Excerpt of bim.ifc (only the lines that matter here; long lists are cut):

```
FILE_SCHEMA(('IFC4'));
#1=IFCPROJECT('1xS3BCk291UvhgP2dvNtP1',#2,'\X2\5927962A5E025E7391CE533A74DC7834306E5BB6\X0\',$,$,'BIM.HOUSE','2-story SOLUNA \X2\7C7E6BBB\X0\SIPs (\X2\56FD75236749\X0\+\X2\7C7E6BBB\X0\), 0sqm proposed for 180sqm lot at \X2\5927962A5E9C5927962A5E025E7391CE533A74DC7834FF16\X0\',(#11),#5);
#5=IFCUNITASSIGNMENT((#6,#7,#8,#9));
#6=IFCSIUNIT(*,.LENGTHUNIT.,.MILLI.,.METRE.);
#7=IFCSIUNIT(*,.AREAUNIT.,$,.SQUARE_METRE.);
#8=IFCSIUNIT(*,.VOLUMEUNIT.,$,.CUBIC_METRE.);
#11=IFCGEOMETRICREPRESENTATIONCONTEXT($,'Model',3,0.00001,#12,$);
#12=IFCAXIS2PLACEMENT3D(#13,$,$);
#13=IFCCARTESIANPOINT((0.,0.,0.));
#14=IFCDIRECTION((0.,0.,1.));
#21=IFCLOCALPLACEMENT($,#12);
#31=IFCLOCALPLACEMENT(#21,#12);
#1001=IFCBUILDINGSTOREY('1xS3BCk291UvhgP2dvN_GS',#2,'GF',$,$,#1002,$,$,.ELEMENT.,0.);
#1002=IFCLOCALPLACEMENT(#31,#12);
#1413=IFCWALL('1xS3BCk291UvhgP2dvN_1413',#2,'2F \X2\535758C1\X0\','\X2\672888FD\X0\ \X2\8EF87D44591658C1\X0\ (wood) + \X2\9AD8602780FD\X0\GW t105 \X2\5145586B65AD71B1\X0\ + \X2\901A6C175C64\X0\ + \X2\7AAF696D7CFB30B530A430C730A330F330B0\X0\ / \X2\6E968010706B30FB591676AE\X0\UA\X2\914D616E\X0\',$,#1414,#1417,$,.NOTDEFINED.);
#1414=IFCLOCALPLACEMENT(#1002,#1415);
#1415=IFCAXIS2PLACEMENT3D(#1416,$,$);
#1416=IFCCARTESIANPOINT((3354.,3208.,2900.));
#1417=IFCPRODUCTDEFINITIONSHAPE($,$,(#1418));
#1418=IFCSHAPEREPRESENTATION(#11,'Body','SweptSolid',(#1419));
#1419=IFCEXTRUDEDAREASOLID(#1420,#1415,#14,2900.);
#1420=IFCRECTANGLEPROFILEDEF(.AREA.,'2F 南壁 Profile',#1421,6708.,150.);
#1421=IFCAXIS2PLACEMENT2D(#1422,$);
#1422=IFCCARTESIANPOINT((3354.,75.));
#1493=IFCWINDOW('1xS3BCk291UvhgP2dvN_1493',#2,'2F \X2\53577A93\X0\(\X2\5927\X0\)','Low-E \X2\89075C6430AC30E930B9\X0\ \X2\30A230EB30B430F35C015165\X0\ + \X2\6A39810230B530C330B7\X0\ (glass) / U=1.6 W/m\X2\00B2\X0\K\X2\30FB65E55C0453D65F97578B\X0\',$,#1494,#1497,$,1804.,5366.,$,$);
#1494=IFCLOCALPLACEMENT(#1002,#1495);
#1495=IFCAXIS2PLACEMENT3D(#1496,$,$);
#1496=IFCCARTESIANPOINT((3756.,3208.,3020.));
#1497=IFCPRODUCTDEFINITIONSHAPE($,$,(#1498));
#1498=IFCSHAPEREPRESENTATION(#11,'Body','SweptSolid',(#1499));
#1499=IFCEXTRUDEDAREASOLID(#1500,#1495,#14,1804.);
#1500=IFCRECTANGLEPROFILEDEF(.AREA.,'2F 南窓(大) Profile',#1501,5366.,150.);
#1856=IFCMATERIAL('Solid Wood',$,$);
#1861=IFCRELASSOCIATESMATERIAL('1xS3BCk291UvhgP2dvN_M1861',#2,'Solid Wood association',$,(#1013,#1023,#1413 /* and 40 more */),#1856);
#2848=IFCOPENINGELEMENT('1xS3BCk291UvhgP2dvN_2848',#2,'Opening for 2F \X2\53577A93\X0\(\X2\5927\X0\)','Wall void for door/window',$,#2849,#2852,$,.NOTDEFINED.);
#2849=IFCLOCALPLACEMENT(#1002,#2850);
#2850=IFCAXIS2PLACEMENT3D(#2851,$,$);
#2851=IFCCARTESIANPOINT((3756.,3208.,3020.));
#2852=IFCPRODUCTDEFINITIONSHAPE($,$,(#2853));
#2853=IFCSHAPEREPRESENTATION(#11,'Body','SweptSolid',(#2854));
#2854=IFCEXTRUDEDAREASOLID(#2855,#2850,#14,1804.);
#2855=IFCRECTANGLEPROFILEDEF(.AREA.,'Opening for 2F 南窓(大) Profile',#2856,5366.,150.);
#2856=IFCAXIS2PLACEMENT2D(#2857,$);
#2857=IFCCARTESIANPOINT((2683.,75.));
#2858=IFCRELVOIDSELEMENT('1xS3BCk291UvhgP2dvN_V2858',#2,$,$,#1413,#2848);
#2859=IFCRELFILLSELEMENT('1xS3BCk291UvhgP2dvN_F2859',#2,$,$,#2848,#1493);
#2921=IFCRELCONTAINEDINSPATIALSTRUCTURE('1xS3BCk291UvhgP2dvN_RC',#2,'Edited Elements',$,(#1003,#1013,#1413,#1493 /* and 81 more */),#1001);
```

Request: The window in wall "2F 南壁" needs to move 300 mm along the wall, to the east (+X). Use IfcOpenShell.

```python
import ifcopenshell
import ifcopenshell.api.geometry
import ifcopenshell.util.placement
import ifcopenshell.util.unit

model = ifcopenshell.open("bim.ifc")
unit_scale = ifcopenshell.util.unit.calculate_unit_scale(model)

window = model.by_guid("1xS3BCk291UvhgP2dvN_1493")
opening = window.FillsVoids[0].RelatingOpeningElement
wall = opening.VoidsElements[0].RelatingBuildingElement

wall_matrix = ifcopenshell.util.placement.get_local_placement(wall.ObjectPlacement)
shift = wall_matrix[:3, 0] * 0.3 / unit_scale
before = ifcopenshell.util.placement.get_local_placement(window.ObjectPlacement)[:3, 3].copy()

# The window is not placed relative to its opening, so move both.
for product in (opening, window):
    matrix = ifcopenshell.util.placement.get_local_placement(product.ObjectPlacement)
    matrix[:3, 3] += shift
    ifcopenshell.api.geometry.edit_object_placement(model, product=product, matrix=matrix, is_si=False)

after = ifcopenshell.util.placement.get_local_placement(window.ObjectPlacement)[:3, 3]
print("window moved by", (after - before).round(3) + 0.0)

model.write("bim_updated.ifc")
```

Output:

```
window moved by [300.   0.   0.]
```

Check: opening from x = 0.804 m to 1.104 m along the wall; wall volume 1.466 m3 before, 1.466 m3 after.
